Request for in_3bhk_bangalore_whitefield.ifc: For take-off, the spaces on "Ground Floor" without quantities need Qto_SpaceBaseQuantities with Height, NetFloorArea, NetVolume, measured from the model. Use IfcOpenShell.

First a look at what the model holds.

```python
import ifcopenshell
import ifcopenshell.util.element
import ifcopenshell.util.unit

model = ifcopenshell.open("in_3bhk_bangalore_whitefield.ifc")
print(model.schema)
for unit_type in ("LENGTHUNIT", "AREAUNIT", "VOLUMEUNIT"):
    print(unit_type, ifcopenshell.util.unit.calculate_unit_scale(model, unit_type))
storey = next(s for s in model.by_type("IfcBuildingStorey") if s.Name == "Ground Floor")
spaces = [e for e in ifcopenshell.util.element.get_decomposition(storey) if e.is_a("IfcSpace")]
for e in sorted(spaces, key=lambda e: e.id()):
    print(e.id(), e.is_a(), e.Name, list(ifcopenshell.util.element.get_psets(e, qtos_only=True)), sep=" | ")
```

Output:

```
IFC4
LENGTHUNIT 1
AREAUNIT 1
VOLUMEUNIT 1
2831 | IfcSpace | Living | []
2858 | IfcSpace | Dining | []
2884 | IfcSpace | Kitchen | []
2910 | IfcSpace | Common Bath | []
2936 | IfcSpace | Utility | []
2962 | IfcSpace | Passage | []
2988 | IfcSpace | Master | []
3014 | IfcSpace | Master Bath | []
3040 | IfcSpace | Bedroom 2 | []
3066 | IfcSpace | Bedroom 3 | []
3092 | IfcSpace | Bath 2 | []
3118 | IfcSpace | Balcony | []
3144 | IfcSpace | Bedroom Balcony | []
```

```python
import ifcopenshell
import ifcopenshell.api.pset
import ifcopenshell.geom
import ifcopenshell.util.element
import ifcopenshell.util.shape
import ifcopenshell.util.unit

model = ifcopenshell.open("in_3bhk_bangalore_whitefield.ifc")
unit_scale = ifcopenshell.util.unit.calculate_unit_scale(model)
area_scale = ifcopenshell.util.unit.calculate_unit_scale(model, "AREAUNIT")
volume_scale = ifcopenshell.util.unit.calculate_unit_scale(model, "VOLUMEUNIT")
settings = ifcopenshell.geom.settings()

storey = next(s for s in model.by_type("IfcBuildingStorey") if s.Name == "Ground Floor")
spaces = [e for e in ifcopenshell.util.element.get_decomposition(storey) if e.is_a("IfcSpace")]

for e in sorted(spaces, key=lambda e: e.id()):
    if ifcopenshell.util.element.get_psets(e, qtos_only=True, should_inherit=False):
        continue
    # Geometry comes back in metres, in the element's own axes.
    shape = ifcopenshell.geom.create_shape(settings, e)
    values = {
        "Height": ifcopenshell.util.shape.get_z(shape.geometry) / unit_scale,
        "NetFloorArea": ifcopenshell.util.shape.get_footprint_area(shape.geometry) / area_scale,
        "NetVolume": ifcopenshell.util.shape.get_volume(shape.geometry) / volume_scale,
    }
    qto = ifcopenshell.api.pset.add_qto(model, product=e, name="Qto_SpaceBaseQuantities")
    ifcopenshell.api.pset.edit_qto(model, qto=qto, properties=values)
    print(e.id(), {k: round(v, 3) for k, v in values.items()})

model.write("in_3bhk_bangalore_whitefield_v2.ifc")
```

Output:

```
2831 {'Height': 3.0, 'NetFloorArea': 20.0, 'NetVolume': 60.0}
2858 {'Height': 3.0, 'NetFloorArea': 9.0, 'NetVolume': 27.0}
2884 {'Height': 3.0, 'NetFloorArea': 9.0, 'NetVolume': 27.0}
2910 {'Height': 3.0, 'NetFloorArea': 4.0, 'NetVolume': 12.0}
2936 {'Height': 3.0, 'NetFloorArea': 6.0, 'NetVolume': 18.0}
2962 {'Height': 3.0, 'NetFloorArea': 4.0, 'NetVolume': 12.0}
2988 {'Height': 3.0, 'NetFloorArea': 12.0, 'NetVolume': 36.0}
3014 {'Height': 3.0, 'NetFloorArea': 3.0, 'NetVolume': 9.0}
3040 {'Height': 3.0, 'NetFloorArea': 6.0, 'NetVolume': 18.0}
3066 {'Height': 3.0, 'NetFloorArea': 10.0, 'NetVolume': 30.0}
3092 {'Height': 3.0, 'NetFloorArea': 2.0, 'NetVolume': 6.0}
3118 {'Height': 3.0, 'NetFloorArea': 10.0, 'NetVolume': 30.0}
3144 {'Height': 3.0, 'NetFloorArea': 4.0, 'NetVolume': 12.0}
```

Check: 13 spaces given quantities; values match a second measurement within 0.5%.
